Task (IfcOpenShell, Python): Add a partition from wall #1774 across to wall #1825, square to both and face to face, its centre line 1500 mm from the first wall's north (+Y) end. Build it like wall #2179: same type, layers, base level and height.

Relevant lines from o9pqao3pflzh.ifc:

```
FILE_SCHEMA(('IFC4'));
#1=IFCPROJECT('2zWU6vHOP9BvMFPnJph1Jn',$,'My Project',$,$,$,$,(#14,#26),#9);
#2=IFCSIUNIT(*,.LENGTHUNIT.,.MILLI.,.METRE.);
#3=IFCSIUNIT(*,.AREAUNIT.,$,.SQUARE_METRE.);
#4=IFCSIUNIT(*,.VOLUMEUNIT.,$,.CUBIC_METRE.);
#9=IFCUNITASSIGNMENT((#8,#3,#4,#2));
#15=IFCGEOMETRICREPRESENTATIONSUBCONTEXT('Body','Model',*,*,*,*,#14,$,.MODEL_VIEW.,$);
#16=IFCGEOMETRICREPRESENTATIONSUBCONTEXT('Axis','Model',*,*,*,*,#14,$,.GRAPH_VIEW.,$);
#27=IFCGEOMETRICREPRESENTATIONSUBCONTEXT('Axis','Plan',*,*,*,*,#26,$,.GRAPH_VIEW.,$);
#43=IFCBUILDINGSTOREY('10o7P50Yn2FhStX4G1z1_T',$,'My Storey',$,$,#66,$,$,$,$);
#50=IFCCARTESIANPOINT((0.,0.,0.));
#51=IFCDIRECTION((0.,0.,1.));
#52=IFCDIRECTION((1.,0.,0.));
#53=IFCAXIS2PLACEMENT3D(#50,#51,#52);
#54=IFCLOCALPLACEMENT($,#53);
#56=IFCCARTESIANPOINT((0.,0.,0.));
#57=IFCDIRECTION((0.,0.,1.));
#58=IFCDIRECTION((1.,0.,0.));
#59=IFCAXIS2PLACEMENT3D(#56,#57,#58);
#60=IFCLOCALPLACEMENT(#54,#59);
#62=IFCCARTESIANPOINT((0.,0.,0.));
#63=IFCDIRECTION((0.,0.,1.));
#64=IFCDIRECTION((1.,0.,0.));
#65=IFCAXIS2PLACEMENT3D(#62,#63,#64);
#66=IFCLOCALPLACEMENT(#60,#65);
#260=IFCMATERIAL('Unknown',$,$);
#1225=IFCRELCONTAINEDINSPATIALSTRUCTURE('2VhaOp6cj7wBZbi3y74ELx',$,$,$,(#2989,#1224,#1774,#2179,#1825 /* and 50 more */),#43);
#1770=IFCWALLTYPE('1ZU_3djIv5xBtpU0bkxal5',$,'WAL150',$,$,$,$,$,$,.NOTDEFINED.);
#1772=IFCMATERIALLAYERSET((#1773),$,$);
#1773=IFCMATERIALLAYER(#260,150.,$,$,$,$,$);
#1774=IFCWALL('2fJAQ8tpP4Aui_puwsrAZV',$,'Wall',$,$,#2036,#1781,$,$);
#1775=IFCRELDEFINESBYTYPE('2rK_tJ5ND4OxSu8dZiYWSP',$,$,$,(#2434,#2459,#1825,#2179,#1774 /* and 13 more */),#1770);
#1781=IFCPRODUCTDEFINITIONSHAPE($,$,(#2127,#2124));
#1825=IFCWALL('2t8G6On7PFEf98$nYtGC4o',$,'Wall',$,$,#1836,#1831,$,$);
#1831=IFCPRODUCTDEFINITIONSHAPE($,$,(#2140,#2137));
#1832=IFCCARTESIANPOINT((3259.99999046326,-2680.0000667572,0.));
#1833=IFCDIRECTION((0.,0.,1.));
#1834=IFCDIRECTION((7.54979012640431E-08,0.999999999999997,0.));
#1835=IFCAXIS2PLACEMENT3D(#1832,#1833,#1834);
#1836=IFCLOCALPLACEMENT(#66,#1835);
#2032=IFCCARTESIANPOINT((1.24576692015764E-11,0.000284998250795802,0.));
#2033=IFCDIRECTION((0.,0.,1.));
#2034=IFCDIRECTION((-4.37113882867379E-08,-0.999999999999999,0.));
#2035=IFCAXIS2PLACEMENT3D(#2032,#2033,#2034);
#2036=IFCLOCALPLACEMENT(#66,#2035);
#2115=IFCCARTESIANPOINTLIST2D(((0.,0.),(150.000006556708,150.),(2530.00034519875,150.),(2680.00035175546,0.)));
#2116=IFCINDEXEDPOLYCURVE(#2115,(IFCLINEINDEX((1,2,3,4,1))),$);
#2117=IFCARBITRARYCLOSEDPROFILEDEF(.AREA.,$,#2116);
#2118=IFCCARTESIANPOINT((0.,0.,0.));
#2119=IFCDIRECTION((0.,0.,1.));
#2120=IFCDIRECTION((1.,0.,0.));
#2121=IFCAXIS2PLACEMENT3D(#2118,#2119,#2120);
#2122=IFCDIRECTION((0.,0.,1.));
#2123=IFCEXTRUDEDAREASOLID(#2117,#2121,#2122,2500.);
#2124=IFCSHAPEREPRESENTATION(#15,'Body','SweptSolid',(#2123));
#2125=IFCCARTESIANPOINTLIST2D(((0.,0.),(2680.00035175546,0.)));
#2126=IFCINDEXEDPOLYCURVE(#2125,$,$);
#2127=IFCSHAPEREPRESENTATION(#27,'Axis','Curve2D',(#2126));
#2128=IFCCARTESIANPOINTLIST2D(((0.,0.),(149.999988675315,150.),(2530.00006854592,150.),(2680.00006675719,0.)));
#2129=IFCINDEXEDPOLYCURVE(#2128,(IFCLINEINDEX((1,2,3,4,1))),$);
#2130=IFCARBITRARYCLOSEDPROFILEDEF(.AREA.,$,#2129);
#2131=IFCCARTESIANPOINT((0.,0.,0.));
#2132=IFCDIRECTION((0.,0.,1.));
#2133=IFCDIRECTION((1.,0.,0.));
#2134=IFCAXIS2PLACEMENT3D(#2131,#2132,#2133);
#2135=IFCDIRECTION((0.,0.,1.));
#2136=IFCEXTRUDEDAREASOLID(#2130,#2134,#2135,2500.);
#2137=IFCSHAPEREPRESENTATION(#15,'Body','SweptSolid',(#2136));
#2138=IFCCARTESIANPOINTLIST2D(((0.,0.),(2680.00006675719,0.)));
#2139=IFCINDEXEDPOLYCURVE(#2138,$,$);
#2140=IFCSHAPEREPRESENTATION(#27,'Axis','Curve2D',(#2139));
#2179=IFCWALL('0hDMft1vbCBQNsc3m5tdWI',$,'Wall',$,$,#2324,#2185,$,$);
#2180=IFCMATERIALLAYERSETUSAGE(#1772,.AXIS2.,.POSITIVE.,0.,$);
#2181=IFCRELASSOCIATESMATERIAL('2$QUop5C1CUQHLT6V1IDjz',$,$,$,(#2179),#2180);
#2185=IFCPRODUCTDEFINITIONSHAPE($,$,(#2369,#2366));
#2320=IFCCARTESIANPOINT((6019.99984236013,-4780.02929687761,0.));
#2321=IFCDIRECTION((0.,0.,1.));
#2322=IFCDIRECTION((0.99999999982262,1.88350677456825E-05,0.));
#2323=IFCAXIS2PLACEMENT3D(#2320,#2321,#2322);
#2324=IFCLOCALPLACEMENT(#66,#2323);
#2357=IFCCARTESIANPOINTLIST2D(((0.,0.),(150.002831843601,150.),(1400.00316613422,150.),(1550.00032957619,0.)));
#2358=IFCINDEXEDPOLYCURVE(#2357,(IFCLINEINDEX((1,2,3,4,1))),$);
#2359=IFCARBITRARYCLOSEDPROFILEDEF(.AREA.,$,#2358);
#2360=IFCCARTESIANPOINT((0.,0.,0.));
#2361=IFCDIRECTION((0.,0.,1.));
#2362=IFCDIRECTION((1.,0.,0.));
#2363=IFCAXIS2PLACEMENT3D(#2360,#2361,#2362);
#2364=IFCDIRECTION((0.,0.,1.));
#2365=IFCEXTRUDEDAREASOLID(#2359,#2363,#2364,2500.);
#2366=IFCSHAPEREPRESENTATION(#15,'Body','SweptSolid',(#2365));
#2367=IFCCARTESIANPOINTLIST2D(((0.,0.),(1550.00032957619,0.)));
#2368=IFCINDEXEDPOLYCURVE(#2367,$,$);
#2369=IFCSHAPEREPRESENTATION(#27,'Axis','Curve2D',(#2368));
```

```python
import numpy as np
import ifcopenshell
import ifcopenshell.api.geometry
import ifcopenshell.api.material
import ifcopenshell.api.pset
import ifcopenshell.api.root
import ifcopenshell.api.spatial
import ifcopenshell.api.type
import ifcopenshell.geom
import ifcopenshell.util.element
import ifcopenshell.util.placement
import ifcopenshell.util.representation
import ifcopenshell.util.shape
import ifcopenshell.util.unit

model = ifcopenshell.open("o9pqao3pflzh.ifc")
unit_scale = ifcopenshell.util.unit.calculate_unit_scale(model)
settings = ifcopenshell.geom.settings()
settings.set("use-world-coords", True)

start_wall = model.by_guid("2fJAQ8tpP4Aui_puwsrAZV")
end_wall = model.by_guid("2t8G6On7PFEf98$nYtGC4o")
like = model.by_guid("0hDMft1vbCBQNsc3m5tdWI")
matrix = ifcopenshell.util.placement.get_local_placement(start_wall.ObjectPlacement)
matrix[:3, 3] *= unit_scale


def extent(element):
    """Bounding box in the first wall's axes, in metres."""
    shape = ifcopenshell.geom.create_shape(settings, element)
    points = (ifcopenshell.util.shape.get_vertices(shape.geometry) - matrix[:3, 3]) @ matrix[:3, :3]
    return points.min(axis=0), points.max(axis=0)


y_start = extent(start_wall)[1][1]
y_end = extent(end_wall)[0][1]
like_min, like_max = extent(like)
length, height = float(abs(y_end - y_start)), float(like_max[2] - like_min[2])
layer_set = ifcopenshell.util.element.get_material(like, should_skip_usage=True)
thickness = sum(layer.LayerThickness for layer in layer_set.MaterialLayers) * unit_scale

wall = ifcopenshell.api.root.create_entity(model, ifc_class="IfcWall", name="New partition")
storey = ifcopenshell.util.element.get_container(like)
ifcopenshell.api.spatial.assign_container(model, products=[wall], relating_structure=storey)
ifcopenshell.api.type.assign_type(
    model, related_objects=[wall], relating_type=ifcopenshell.util.element.get_type(like), should_map_representations=False
)
rel = ifcopenshell.api.material.assign_material(
    model, products=[wall], type="IfcMaterialLayerSetUsage", material=layer_set
)
rel.RelatingMaterial.OffsetFromReferenceLine = -thickness / 2 / unit_scale
pset = ifcopenshell.api.pset.add_pset(model, product=wall, name="Pset_WallCommon")
ifcopenshell.api.pset.edit_pset(model, pset=pset, properties={"IsExternal": False, "LoadBearing": False})

# The axis runs down the middle of the wall.
axis = ifcopenshell.api.geometry.add_axis_representation(
    model, context=ifcopenshell.util.representation.get_context(model, "Model", "Axis"), axis=[(0.0, 0.0), (length, 0.0)]
)
body = ifcopenshell.api.geometry.add_wall_representation(
    model,
    context=ifcopenshell.util.representation.get_context(model, "Model", "Body", "MODEL_VIEW"),
    length=length,
    height=height,
    thickness=thickness,
    offset=-thickness / 2,
)
for representation in (axis, body):
    ifcopenshell.api.geometry.assign_representation(model, product=wall, representation=representation)

placement = matrix @ ifcopenshell.util.placement.rotation(90, "Z")
placement[:, 3] = matrix @ np.array([extent(start_wall)[0][0] + 1.5, y_start, like_min[2], 1.0])
ifcopenshell.api.geometry.edit_object_placement(model, product=wall, matrix=placement)

print(f"partition {length:.3f} m long, {height:.3f} m high, {thickness:.3f} m thick")

model.write("o9pqao3pflzh-out.ifc")
```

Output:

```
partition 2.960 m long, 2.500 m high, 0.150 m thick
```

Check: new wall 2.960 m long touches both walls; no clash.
